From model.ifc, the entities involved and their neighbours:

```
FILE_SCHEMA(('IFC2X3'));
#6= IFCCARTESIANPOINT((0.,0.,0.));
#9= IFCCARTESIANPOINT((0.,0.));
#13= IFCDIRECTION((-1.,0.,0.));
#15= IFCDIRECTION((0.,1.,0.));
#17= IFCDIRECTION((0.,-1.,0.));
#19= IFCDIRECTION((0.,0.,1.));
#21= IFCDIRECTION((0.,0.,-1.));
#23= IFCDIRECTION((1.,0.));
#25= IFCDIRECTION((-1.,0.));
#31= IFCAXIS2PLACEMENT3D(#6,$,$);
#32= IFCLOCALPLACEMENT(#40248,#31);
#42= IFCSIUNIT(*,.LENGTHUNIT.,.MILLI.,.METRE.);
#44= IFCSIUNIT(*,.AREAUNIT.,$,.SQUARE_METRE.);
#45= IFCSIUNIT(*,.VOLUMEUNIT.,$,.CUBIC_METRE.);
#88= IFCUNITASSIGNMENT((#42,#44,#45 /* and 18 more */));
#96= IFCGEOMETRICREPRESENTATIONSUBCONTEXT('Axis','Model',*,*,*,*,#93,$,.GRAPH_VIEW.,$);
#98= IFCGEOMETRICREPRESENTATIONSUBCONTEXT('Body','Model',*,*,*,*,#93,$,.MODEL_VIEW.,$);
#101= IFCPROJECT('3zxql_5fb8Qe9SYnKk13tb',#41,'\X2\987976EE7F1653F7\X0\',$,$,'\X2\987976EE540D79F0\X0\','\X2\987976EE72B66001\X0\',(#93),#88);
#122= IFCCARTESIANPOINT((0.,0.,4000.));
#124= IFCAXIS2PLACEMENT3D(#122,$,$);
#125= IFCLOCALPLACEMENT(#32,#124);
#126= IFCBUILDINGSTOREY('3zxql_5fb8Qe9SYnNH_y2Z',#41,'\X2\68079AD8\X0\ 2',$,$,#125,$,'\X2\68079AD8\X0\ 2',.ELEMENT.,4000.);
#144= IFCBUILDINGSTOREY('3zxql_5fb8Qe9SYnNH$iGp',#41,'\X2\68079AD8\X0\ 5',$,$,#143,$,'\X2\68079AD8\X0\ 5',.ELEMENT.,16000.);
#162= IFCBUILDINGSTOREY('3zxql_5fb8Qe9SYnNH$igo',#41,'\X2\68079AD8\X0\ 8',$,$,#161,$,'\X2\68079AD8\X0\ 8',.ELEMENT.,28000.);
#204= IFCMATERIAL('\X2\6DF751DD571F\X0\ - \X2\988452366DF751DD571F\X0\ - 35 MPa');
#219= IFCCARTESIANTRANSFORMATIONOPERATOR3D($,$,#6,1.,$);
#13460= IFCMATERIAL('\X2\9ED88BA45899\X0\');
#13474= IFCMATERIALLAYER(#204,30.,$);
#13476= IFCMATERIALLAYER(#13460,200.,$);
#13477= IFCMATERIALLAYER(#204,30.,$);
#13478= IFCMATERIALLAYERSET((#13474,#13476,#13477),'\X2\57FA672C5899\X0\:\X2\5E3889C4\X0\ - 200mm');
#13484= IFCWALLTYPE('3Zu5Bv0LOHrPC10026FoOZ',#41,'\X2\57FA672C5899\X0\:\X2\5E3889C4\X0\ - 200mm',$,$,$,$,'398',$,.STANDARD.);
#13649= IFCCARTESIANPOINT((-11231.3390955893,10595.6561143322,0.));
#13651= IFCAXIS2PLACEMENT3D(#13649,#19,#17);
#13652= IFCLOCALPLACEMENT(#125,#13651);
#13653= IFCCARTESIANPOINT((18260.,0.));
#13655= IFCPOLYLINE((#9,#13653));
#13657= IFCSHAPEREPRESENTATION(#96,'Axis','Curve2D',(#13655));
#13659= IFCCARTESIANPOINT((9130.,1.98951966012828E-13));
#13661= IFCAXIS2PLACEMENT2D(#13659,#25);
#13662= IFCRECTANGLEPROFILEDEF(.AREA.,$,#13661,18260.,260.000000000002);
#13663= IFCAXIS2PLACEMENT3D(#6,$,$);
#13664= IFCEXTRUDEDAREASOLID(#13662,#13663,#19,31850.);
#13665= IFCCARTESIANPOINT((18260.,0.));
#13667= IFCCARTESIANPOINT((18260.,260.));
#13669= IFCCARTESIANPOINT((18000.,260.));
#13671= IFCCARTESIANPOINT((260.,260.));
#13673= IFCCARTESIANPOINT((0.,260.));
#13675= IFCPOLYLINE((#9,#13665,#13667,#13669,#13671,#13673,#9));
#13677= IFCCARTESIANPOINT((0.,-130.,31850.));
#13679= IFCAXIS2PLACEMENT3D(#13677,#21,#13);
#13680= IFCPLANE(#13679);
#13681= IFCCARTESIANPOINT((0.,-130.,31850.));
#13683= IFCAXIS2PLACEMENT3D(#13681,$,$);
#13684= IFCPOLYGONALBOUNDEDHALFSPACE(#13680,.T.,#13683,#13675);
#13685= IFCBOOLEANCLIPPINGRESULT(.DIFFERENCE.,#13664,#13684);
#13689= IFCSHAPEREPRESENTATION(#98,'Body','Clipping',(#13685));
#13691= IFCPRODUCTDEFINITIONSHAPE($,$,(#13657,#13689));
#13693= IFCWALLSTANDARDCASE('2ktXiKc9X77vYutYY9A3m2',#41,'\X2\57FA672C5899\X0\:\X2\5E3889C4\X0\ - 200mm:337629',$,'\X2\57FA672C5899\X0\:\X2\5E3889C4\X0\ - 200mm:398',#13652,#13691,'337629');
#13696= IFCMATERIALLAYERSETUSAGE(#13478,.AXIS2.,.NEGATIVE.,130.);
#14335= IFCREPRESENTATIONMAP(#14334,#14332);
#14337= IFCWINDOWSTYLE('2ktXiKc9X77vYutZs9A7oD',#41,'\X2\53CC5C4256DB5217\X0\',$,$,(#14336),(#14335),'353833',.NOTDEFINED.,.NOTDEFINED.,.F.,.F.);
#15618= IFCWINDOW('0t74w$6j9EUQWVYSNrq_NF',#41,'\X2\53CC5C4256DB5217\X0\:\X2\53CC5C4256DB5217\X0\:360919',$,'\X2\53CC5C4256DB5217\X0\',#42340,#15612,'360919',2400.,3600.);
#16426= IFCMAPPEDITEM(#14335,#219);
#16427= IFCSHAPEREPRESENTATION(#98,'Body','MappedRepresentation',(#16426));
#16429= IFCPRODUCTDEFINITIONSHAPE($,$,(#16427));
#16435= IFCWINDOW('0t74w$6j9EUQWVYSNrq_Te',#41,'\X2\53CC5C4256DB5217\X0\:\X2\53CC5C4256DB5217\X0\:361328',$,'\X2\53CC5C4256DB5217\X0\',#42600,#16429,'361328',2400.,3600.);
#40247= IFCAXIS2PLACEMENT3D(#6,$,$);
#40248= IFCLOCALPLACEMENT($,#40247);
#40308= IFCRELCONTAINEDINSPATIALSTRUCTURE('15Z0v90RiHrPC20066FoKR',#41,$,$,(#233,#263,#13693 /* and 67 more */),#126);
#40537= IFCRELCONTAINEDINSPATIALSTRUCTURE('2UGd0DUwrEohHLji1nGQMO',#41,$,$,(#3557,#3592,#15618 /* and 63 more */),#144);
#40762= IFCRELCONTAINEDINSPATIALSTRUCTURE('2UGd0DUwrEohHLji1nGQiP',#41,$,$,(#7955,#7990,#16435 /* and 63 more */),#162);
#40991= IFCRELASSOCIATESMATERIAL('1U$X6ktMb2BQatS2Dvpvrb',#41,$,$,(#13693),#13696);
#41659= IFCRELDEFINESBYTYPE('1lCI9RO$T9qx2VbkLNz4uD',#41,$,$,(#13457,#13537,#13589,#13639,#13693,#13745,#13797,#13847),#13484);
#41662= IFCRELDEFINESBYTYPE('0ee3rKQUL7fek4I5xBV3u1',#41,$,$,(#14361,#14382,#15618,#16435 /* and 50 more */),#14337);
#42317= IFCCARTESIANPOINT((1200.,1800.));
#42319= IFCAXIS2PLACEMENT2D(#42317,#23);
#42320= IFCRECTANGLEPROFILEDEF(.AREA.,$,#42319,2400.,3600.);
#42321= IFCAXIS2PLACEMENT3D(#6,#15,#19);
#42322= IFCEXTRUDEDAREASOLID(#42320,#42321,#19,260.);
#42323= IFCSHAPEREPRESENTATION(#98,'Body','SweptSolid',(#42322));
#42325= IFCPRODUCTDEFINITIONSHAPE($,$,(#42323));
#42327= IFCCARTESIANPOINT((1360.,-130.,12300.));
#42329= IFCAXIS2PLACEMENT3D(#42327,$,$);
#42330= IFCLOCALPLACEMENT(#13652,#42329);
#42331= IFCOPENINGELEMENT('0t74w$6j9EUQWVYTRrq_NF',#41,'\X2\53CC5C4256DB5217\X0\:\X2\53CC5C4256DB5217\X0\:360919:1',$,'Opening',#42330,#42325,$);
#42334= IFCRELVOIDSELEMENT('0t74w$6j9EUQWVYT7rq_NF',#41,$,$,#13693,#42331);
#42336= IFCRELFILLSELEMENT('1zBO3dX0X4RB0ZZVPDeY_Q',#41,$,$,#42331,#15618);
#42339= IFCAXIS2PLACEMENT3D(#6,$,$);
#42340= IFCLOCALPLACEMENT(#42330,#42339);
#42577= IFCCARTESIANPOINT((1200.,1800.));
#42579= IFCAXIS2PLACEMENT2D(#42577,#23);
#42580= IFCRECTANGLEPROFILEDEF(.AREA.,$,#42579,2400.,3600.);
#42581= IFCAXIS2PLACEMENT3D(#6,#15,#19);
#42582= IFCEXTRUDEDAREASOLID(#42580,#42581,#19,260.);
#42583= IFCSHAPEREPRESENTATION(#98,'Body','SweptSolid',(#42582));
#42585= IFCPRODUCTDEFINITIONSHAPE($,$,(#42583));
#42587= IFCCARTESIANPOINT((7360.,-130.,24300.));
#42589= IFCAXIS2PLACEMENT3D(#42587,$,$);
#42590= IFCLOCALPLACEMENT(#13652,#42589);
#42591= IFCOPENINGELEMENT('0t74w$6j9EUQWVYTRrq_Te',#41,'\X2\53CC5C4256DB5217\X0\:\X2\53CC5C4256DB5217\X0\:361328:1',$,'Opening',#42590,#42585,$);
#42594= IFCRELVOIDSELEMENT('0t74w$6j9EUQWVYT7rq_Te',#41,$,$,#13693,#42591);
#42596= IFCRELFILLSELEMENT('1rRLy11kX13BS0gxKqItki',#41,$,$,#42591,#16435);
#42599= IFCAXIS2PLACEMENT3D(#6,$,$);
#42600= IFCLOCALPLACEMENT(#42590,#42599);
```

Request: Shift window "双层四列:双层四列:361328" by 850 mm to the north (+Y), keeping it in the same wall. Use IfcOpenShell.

```python
import ifcopenshell
import ifcopenshell.api.geometry
import ifcopenshell.util.placement
import ifcopenshell.util.unit

model = ifcopenshell.open("model.ifc")
unit_scale = ifcopenshell.util.unit.calculate_unit_scale(model)

window = model.by_guid("0t74w$6j9EUQWVYSNrq_Te")
opening = window.FillsVoids[0].RelatingOpeningElement
wall = opening.VoidsElements[0].RelatingBuildingElement

wall_matrix = ifcopenshell.util.placement.get_local_placement(wall.ObjectPlacement)
shift = wall_matrix[:3, 0] * -0.85 / unit_scale
before = ifcopenshell.util.placement.get_local_placement(window.ObjectPlacement)[:3, 3].copy()

# The window is placed relative to its opening, so it follows when the opening moves.
matrix = ifcopenshell.util.placement.get_local_placement(opening.ObjectPlacement)
matrix[:3, 3] += shift
ifcopenshell.api.geometry.edit_object_placement(
    model, product=opening, matrix=matrix, is_si=False, should_transform_children=True
)

after = ifcopenshell.util.placement.get_local_placement(window.ObjectPlacement)[:3, 3]
print("window moved by", (after - before).round(3) + 0.0)

model.write("model_updated.ifc")
```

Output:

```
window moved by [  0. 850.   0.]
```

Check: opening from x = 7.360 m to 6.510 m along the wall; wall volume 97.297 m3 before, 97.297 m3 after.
